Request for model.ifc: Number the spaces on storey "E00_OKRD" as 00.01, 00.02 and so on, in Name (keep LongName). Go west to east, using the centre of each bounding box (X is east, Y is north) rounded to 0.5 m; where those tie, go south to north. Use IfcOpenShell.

First a look at what the model holds.

```python
import ifcopenshell
import ifcopenshell.util.element
import ifcopenshell.util.placement

model = ifcopenshell.open("model.ifc")
print(model.schema)
storey = next(s for s in model.by_type("IfcBuildingStorey") if s.Name == "E00_OKRD")
spaces = [e for e in ifcopenshell.util.element.get_decomposition(storey) if e.is_a("IfcSpace")]
for e in sorted(spaces, key=lambda e: e.id()):
    origin = ifcopenshell.util.placement.get_local_placement(e.ObjectPlacement)[:3, 3]
    print(e.id(), e.Name, e.LongName, origin.round(2) + 0.0, sep=" | ")
```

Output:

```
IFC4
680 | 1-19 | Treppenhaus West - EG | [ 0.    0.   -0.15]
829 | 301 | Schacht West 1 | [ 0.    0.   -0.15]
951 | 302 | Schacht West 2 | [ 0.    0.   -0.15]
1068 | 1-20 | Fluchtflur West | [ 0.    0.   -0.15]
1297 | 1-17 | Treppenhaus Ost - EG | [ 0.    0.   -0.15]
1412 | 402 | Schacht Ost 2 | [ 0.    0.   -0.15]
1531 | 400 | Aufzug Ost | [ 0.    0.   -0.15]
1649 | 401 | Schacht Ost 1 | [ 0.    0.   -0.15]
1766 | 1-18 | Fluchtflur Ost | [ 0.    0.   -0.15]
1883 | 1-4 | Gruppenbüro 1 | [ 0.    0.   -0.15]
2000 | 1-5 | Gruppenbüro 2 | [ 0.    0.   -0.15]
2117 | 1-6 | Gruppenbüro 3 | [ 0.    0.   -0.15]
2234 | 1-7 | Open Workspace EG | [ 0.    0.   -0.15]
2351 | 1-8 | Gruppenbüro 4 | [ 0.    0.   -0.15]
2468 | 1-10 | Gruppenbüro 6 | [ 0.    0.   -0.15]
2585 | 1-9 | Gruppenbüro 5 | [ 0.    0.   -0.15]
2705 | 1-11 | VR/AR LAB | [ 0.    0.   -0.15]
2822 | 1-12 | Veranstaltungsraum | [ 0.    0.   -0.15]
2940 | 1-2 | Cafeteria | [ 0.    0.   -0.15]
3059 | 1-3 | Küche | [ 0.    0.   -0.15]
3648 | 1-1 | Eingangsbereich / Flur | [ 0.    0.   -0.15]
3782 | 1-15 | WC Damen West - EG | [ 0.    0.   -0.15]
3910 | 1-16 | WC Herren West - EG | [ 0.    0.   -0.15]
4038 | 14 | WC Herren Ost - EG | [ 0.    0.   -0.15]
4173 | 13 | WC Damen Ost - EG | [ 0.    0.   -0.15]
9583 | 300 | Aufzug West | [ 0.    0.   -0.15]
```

```python
import ifcopenshell
import ifcopenshell.geom
import ifcopenshell.util.element
import ifcopenshell.util.shape

model = ifcopenshell.open("model.ifc")
settings = ifcopenshell.geom.settings()
settings.set("use-world-coords", True)


def centre(element):
    shape = ifcopenshell.geom.create_shape(settings, element)
    return ifcopenshell.util.shape.get_bbox_centroid(shape.geometry)


storey = next(s for s in model.by_type("IfcBuildingStorey") if s.Name == "E00_OKRD")
spaces = [e for e in ifcopenshell.util.element.get_decomposition(storey) if e.is_a("IfcSpace")]

# Insertion points can sit at a corner or the storey origin, so sort by the geometry (in metres).
centres = {e: centre(e) for e in spaces}
spaces.sort(key=lambda e: (round(centres[e][0] / 0.5), centres[e][1]))

for i, e in enumerate(spaces, start=1):
    number = f"00.{i:02d}"
    e.Name = number
    print(e.id(), number)

model.write("model_rev.ifc")
```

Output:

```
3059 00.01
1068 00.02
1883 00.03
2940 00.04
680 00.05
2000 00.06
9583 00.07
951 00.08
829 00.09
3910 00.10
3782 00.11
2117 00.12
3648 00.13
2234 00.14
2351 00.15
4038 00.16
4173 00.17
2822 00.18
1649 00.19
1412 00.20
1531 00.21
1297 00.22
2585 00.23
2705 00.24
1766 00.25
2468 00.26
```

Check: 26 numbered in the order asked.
